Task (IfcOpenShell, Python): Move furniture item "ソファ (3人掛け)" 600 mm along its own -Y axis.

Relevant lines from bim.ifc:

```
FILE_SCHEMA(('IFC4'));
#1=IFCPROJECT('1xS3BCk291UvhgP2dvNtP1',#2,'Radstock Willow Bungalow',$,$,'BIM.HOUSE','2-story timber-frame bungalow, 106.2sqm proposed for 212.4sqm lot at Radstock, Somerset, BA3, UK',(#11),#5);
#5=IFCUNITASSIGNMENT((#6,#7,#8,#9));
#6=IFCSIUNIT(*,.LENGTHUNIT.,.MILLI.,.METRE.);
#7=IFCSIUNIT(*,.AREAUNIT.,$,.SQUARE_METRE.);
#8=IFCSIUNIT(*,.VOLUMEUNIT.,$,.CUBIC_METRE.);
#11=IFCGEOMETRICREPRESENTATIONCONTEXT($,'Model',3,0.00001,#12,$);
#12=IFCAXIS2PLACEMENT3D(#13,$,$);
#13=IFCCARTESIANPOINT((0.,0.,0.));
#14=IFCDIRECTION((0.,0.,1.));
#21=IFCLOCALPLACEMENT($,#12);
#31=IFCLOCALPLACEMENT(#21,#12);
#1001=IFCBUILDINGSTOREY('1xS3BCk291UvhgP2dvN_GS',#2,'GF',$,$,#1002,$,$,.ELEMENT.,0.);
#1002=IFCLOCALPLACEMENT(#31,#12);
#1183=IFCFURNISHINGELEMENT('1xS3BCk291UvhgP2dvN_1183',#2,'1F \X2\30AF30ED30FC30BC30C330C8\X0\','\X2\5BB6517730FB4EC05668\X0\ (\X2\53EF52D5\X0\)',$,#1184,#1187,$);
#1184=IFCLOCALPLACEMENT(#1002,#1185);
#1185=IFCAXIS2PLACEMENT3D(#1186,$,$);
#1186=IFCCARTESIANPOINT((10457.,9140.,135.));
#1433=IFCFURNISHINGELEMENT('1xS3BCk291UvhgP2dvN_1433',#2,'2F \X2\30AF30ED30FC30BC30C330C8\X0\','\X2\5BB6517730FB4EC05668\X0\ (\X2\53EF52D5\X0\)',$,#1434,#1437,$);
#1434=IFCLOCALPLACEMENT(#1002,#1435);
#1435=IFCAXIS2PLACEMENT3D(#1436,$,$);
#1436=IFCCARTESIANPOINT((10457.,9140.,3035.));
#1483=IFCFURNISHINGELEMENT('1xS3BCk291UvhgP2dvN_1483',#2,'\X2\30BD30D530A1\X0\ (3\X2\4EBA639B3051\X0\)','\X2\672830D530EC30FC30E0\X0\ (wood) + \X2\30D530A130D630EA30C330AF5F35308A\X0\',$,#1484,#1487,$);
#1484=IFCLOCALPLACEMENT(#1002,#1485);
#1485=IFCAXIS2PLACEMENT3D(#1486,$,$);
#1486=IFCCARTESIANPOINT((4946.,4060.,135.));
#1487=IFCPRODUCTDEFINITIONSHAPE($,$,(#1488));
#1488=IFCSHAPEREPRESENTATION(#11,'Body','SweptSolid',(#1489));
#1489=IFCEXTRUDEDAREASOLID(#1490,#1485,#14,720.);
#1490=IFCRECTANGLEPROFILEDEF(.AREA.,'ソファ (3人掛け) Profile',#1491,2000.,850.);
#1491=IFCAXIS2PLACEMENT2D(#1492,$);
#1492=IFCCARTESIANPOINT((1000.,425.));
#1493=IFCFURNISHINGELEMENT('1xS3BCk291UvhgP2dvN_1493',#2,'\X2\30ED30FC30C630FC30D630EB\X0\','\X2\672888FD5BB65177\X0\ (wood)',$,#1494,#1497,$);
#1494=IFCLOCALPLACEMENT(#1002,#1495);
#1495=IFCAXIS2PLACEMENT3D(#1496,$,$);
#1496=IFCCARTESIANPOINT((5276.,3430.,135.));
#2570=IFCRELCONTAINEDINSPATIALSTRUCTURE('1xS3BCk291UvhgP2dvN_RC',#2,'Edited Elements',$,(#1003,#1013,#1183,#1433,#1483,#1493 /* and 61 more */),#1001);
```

```python
import ifcopenshell
import ifcopenshell.api.geometry
import ifcopenshell.util.placement
import ifcopenshell.util.unit

model = ifcopenshell.open("bim.ifc")
unit_scale = ifcopenshell.util.unit.calculate_unit_scale(model)

item = model.by_guid("1xS3BCk291UvhgP2dvN_1483")
matrix = ifcopenshell.util.placement.get_local_placement(item.ObjectPlacement)
matrix[:3, 3] -= matrix[:3, 1] * 0.6 / unit_scale
ifcopenshell.api.geometry.edit_object_placement(model, product=item, matrix=matrix, is_si=False)

print(ifcopenshell.util.placement.get_local_placement(item.ObjectPlacement).round(3) + 0.0)

model.write("bim-out.ifc")
```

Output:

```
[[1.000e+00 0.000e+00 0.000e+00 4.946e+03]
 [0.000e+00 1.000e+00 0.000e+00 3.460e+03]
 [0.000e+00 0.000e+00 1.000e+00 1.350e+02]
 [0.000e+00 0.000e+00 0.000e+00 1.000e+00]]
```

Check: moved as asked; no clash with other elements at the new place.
